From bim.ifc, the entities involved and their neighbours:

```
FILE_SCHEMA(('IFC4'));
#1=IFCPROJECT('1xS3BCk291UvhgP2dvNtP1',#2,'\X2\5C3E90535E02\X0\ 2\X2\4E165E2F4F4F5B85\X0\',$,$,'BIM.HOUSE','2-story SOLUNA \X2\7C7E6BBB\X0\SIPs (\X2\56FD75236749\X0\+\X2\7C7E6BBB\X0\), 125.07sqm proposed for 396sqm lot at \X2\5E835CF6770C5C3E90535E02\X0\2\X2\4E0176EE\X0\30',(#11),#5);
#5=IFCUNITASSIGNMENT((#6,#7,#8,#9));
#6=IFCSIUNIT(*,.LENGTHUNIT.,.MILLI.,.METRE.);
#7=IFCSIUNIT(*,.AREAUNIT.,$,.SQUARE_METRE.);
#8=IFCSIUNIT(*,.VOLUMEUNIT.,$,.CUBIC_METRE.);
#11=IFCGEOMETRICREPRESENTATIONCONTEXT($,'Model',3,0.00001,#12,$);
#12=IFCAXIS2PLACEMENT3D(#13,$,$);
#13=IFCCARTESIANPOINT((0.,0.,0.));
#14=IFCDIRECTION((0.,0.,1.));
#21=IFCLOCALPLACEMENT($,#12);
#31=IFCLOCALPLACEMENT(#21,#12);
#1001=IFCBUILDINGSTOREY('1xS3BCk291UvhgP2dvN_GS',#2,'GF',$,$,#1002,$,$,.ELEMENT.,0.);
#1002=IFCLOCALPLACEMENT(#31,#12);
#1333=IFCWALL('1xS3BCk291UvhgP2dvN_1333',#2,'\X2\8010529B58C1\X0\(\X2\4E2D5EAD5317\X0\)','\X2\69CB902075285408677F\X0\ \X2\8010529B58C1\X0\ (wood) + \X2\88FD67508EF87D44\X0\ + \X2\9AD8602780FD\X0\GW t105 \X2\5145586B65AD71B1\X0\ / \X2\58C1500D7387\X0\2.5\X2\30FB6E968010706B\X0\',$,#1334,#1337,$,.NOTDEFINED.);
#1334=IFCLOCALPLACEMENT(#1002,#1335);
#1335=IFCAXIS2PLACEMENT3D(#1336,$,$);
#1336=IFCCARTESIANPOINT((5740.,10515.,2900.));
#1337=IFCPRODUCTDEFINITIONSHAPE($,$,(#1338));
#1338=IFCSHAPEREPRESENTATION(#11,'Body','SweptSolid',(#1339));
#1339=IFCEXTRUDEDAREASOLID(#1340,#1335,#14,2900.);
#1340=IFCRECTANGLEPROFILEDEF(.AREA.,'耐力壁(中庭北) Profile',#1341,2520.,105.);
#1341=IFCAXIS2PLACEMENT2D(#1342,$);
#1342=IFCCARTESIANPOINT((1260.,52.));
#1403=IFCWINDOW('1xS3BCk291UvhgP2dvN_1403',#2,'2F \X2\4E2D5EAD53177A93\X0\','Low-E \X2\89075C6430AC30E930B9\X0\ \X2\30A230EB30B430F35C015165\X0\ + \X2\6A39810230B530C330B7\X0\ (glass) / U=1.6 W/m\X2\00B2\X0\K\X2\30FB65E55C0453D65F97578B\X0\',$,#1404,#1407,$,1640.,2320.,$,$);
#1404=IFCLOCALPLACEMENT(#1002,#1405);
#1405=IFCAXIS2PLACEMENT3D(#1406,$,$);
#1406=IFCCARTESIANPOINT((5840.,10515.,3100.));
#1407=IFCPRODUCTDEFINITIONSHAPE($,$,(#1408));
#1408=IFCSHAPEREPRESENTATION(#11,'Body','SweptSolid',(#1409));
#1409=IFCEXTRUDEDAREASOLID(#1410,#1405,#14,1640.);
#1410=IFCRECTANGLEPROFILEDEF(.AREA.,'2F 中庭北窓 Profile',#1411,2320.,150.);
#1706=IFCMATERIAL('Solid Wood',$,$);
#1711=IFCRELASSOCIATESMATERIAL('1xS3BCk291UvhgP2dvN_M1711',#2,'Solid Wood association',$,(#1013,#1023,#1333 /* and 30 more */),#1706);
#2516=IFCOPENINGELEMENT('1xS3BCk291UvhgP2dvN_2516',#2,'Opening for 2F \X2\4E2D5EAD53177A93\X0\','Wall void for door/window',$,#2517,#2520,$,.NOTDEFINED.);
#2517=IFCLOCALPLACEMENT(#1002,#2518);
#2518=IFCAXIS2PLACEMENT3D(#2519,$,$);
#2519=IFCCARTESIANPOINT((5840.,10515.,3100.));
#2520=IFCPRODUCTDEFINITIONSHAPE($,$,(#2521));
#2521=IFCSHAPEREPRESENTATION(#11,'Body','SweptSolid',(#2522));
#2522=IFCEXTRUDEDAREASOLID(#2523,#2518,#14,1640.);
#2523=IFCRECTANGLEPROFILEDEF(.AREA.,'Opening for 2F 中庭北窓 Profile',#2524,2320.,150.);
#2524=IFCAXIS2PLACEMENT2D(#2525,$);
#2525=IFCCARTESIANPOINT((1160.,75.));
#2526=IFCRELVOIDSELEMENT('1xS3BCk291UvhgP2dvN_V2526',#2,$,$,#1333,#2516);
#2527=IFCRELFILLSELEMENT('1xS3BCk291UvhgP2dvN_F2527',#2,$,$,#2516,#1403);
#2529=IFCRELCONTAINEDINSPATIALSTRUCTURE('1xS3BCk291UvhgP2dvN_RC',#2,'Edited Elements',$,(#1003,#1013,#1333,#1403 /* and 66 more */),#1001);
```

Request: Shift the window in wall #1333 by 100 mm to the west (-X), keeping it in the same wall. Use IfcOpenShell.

```python
import ifcopenshell
import ifcopenshell.api.geometry
import ifcopenshell.util.placement
import ifcopenshell.util.unit

model = ifcopenshell.open("bim.ifc")
unit_scale = ifcopenshell.util.unit.calculate_unit_scale(model)

window = model.by_guid("1xS3BCk291UvhgP2dvN_1403")
opening = window.FillsVoids[0].RelatingOpeningElement
wall = opening.VoidsElements[0].RelatingBuildingElement

wall_matrix = ifcopenshell.util.placement.get_local_placement(wall.ObjectPlacement)
shift = wall_matrix[:3, 0] * -0.1 / unit_scale
before = ifcopenshell.util.placement.get_local_placement(window.ObjectPlacement)[:3, 3].copy()

# The window is not placed relative to its opening, so move both.
for product in (opening, window):
    matrix = ifcopenshell.util.placement.get_local_placement(product.ObjectPlacement)
    matrix[:3, 3] += shift
    ifcopenshell.api.geometry.edit_object_placement(model, product=product, matrix=matrix, is_si=False)

after = ifcopenshell.util.placement.get_local_placement(window.ObjectPlacement)[:3, 3]
print("window moved by", (after - before).round(3) + 0.0)

model.write("bim_updated.ifc")
```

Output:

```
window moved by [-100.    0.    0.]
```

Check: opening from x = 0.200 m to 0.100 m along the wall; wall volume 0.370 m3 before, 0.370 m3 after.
